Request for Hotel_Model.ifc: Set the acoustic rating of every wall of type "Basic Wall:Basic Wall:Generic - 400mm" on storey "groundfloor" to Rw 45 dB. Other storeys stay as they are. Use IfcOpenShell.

First a look at what the model holds.

```python
import ifcopenshell
import ifcopenshell.util.element

model = ifcopenshell.open("Hotel_Model.ifc")
print(model.schema)
storey = next(s for s in model.by_type("IfcBuildingStorey") if s.Name == "groundfloor")
walls = [e for e in ifcopenshell.util.element.get_decomposition(storey) if e.is_a("IfcWall")]
seen = {}
for e in walls:
    element_type = ifcopenshell.util.element.get_type(e)
    key = (element_type.Name if element_type != e and element_type else None, ifcopenshell.util.element.get_pset(e, "Pset_WallCommon", "AcousticRating"))
    seen[key] = seen.get(key, 0) + 1
for (name, value), count in sorted(seen.items(), key=str):
    print(count, "x", name, "|", value)
```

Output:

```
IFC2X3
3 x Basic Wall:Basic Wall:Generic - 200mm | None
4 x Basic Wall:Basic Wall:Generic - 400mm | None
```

```python
import ifcopenshell
import ifcopenshell.api.pset
import ifcopenshell.util.element

model = ifcopenshell.open("Hotel_Model.ifc")

storey = next(s for s in model.by_type("IfcBuildingStorey") if s.Name == "groundfloor")
walls = [e for e in ifcopenshell.util.element.get_decomposition(storey) if e.is_a("IfcWall")]

count = 0
for e in walls:
    element_type = ifcopenshell.util.element.get_type(e)
    if element_type in (None, e) or element_type.Name != "Basic Wall:Basic Wall:Generic - 400mm":
        continue
    # add_pset returns the element's existing set when there is one.
    pset = ifcopenshell.api.pset.add_pset(model, product=e, name="Pset_WallCommon")
    ifcopenshell.api.pset.edit_pset(model, pset=pset, properties={"AcousticRating": "Rw 45 dB"})
    count += 1

print(count, "walls updated")

model.write("Hotel_Model_edited.ifc")
```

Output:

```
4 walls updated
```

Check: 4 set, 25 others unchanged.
